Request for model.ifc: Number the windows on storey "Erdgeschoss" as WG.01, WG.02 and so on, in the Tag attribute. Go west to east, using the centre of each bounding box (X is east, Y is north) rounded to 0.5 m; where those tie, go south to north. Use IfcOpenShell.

First a look at what the model holds.

```python
import ifcopenshell
import ifcopenshell.util.element
import ifcopenshell.util.placement

model = ifcopenshell.open("model.ifc")
print(model.schema)
storey = next(s for s in model.by_type("IfcBuildingStorey") if s.Name == "Erdgeschoss")
windows = [e for e in ifcopenshell.util.element.get_decomposition(storey) if e.is_a("IfcWindow")]
for e in sorted(windows, key=lambda e: e.id()):
    origin = ifcopenshell.util.placement.get_local_placement(e.ObjectPlacement)[:3, 3]
    print(e.id(), e.Tag, e.Name, origin.round(2) + 0.0, sep=" | ")
```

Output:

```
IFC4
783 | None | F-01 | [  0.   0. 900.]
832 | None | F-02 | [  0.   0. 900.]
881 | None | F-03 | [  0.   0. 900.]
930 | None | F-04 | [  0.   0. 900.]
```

```python
import ifcopenshell
import ifcopenshell.geom
import ifcopenshell.util.element
import ifcopenshell.util.shape

model = ifcopenshell.open("model.ifc")
settings = ifcopenshell.geom.settings()
settings.set("use-world-coords", True)


def centre(element):
    shape = ifcopenshell.geom.create_shape(settings, element)
    return ifcopenshell.util.shape.get_bbox_centroid(shape.geometry)


storey = next(s for s in model.by_type("IfcBuildingStorey") if s.Name == "Erdgeschoss")
windows = [e for e in ifcopenshell.util.element.get_decomposition(storey) if e.is_a("IfcWindow")]

# Insertion points can sit at a corner or the storey origin, so sort by the geometry (in metres).
centres = {e: centre(e) for e in windows}
windows.sort(key=lambda e: (round(centres[e][0] / 0.5), centres[e][1]))

for i, e in enumerate(windows, start=1):
    number = f"WG.{i:02d}"
    e.Tag = number
    print(e.id(), number)

model.write("model_rev.ifc")
```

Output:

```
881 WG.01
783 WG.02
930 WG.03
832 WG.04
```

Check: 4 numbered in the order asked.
